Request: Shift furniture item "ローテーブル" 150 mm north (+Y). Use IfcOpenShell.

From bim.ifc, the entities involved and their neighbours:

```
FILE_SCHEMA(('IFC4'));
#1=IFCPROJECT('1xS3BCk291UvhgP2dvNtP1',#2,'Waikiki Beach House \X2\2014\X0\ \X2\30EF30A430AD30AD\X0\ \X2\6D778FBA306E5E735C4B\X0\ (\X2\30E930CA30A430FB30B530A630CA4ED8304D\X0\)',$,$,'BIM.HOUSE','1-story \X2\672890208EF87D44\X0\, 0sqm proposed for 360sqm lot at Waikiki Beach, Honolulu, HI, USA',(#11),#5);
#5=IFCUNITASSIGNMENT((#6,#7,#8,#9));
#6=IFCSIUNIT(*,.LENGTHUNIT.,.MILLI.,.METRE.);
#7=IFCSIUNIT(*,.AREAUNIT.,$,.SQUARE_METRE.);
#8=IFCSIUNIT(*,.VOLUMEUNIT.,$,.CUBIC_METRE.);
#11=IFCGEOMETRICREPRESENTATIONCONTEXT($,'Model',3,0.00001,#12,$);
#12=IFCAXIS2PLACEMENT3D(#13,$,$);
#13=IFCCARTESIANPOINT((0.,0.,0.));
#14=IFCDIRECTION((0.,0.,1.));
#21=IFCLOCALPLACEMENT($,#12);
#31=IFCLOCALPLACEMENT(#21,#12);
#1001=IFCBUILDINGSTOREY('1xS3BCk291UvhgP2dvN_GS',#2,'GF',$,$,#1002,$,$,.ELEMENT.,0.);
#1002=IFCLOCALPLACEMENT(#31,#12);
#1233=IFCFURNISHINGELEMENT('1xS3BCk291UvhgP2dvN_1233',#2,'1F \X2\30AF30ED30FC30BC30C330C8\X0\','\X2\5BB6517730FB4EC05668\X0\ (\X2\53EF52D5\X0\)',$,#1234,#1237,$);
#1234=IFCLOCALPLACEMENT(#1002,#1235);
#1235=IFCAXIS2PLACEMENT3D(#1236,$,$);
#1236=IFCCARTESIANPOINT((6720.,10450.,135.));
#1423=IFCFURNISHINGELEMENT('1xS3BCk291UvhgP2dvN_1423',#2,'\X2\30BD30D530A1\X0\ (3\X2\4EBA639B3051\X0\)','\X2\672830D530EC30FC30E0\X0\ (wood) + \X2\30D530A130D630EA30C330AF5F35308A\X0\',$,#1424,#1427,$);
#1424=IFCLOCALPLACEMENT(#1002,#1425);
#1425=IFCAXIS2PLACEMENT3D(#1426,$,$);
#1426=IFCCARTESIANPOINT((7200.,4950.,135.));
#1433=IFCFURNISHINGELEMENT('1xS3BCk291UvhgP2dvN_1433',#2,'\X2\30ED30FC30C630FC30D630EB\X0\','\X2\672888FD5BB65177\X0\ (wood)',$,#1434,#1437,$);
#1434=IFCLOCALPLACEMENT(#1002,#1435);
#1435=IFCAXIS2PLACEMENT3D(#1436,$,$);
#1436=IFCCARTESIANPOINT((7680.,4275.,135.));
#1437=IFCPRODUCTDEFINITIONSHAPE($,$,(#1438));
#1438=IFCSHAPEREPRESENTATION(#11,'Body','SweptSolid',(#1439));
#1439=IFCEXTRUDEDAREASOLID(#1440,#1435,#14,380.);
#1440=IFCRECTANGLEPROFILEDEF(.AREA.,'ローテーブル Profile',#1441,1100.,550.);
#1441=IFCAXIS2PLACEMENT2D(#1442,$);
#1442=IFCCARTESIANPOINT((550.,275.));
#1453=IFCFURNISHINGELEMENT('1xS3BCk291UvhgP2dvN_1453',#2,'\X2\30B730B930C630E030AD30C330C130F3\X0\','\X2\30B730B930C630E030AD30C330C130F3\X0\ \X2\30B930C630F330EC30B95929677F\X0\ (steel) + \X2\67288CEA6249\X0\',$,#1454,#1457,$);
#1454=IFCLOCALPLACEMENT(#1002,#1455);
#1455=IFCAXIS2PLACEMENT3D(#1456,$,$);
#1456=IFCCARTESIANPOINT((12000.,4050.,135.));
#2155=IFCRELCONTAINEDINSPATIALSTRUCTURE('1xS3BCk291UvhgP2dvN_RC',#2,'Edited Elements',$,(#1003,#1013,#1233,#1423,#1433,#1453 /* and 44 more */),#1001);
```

```python
import ifcopenshell
import ifcopenshell.api.geometry
import ifcopenshell.util.placement

model = ifcopenshell.open("bim.ifc")

item = model.by_id(1433)
matrix = ifcopenshell.util.placement.get_local_placement(item.ObjectPlacement)
matrix[1, 3] += 150.0
ifcopenshell.api.geometry.edit_object_placement(model, product=item, matrix=matrix, is_si=False)

print(ifcopenshell.util.placement.get_local_placement(item.ObjectPlacement).round(3) + 0.0)

model.write("bim_updated.ifc")
```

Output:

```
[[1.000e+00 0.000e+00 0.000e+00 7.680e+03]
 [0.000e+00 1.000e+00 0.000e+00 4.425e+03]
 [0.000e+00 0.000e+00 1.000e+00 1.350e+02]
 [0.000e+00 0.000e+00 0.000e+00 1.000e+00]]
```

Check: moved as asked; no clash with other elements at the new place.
